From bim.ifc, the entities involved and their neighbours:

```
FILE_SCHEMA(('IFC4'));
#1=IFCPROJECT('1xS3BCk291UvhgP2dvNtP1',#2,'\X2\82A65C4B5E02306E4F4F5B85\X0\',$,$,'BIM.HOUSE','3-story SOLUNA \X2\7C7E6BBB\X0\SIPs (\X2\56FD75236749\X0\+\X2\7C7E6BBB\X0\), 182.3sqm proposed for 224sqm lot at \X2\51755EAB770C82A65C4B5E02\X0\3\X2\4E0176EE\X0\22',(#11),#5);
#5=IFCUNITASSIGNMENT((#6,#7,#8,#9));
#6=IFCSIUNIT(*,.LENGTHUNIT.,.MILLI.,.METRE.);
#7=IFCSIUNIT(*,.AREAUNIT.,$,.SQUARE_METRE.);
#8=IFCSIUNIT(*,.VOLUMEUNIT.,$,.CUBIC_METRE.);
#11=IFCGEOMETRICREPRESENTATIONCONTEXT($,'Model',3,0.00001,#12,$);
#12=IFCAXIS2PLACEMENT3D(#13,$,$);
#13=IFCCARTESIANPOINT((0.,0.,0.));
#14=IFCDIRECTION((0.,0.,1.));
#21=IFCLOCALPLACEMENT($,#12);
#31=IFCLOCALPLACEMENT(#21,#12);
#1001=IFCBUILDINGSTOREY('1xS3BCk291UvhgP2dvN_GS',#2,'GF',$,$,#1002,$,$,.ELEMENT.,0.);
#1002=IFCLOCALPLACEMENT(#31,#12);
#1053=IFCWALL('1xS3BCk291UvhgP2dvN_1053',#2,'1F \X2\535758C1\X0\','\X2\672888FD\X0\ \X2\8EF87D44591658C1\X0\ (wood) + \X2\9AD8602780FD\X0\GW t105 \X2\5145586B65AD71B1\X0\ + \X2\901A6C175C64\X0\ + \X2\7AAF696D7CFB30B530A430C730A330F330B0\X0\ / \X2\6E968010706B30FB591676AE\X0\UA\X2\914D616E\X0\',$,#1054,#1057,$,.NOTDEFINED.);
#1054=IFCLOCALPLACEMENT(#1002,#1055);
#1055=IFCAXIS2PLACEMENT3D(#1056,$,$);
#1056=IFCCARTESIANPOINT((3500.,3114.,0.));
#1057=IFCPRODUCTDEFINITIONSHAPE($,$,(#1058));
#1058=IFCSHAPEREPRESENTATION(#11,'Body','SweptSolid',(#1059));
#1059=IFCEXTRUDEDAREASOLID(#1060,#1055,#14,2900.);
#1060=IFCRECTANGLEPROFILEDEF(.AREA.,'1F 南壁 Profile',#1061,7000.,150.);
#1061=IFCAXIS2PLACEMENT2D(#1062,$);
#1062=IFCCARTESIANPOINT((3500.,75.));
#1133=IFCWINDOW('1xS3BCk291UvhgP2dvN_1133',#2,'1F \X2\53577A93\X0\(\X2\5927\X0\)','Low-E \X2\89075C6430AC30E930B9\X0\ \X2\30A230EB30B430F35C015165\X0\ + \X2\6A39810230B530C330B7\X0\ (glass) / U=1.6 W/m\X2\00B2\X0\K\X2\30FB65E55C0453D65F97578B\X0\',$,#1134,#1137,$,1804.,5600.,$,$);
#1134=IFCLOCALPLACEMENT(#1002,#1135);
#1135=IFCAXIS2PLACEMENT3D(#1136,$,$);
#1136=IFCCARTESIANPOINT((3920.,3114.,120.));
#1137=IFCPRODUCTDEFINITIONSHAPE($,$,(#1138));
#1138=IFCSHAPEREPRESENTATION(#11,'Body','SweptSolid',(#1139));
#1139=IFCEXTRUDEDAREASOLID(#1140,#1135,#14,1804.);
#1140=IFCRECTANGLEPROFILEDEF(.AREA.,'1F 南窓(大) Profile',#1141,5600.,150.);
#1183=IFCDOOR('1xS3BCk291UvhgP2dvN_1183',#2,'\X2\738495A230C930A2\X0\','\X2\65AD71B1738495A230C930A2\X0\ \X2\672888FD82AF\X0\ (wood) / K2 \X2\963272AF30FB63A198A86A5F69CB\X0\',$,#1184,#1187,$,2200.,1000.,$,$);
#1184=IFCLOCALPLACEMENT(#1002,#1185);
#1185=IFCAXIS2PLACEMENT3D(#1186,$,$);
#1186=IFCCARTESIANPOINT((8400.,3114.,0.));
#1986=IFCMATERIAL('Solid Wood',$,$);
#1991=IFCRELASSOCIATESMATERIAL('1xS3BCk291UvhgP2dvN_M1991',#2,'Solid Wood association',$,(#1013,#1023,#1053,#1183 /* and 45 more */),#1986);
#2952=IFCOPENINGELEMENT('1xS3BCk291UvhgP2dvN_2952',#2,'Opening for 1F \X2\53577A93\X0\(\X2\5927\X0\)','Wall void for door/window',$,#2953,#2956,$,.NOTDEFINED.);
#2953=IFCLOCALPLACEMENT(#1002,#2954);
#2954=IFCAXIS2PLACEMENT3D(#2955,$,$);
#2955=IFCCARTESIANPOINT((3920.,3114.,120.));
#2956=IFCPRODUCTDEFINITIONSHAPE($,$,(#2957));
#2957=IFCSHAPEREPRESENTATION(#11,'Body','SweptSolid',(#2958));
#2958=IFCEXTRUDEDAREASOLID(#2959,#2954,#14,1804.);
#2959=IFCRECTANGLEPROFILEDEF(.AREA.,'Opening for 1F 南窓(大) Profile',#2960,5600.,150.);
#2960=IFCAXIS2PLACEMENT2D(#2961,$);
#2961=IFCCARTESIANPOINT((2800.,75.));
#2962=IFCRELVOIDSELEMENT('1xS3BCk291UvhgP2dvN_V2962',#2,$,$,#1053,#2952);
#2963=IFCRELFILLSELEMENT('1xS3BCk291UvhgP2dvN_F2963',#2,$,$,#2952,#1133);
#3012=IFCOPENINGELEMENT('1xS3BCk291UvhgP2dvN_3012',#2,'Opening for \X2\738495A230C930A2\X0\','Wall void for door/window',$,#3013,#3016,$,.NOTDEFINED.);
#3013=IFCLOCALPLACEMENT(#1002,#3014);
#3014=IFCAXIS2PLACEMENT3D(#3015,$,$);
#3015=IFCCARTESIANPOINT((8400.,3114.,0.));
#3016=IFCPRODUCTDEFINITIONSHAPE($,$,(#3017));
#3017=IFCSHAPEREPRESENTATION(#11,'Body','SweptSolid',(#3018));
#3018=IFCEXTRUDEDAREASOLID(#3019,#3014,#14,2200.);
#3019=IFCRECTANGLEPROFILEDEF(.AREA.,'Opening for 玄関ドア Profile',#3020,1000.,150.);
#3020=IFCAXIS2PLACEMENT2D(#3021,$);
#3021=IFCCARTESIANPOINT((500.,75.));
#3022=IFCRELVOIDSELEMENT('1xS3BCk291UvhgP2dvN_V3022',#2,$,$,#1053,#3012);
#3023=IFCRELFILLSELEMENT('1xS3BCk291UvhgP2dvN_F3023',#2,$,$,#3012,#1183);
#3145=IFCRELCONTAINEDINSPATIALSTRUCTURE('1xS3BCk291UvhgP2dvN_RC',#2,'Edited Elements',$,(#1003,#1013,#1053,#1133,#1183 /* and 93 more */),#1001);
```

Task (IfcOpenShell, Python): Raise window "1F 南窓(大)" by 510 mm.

```python
import numpy as np
import ifcopenshell
import ifcopenshell.api.geometry
import ifcopenshell.util.placement
import ifcopenshell.util.unit

model = ifcopenshell.open("bim.ifc")
unit_scale = ifcopenshell.util.unit.calculate_unit_scale(model)

window = model.by_guid("1xS3BCk291UvhgP2dvN_1133")
opening = window.FillsVoids[0].RelatingOpeningElement
dz = 0.51 / unit_scale

shift = np.array([0.0, 0.0, dz])
# The window is not placed relative to its opening, so move both.
for product in (opening, window):
    matrix = ifcopenshell.util.placement.get_local_placement(product.ObjectPlacement)
    matrix[:3, 3] += shift
    ifcopenshell.api.geometry.edit_object_placement(model, product=product, matrix=matrix, is_si=False)

print(f"moved by {dz * unit_scale:+.3f} m")

model.write("bim_v2.ifc")
```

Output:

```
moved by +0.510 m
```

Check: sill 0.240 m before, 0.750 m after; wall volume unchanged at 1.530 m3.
